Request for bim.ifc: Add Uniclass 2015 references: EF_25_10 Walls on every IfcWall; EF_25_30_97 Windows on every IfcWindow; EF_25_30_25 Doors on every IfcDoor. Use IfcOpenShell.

First a look at what the model holds.

```python
import ifcopenshell

model = ifcopenshell.open("bim.ifc")
print(model.schema)
print("classifications:", [c.Name for c in model.by_type("IfcClassification")])
for ifc_class in ("IfcDoor", "IfcRoof", "IfcStair", "IfcWall", "IfcWindow"):
    print(ifc_class, len(model.by_type(ifc_class)))
```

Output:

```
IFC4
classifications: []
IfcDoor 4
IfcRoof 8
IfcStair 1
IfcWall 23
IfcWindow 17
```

```python
import ifcopenshell
import ifcopenshell.api.classification

model = ifcopenshell.open("bim.ifc")

system = ifcopenshell.api.classification.add_classification(model, classification="Uniclass 2015")

codes = {
    "IfcWall": ("EF_25_10", "Walls"),
    "IfcWindow": ("EF_25_30_97", "Windows"),
    "IfcDoor": ("EF_25_30_25", "Doors"),
}
for ifc_class, (code, name) in codes.items():
    products = model.by_type(ifc_class)
    ifcopenshell.api.classification.add_reference(
        model, products=products, classification=system, identification=code, name=name
    )
    print(code, len(products))

model.write("bim-out.ifc")
```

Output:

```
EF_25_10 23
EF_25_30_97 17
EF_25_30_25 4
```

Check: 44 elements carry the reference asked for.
